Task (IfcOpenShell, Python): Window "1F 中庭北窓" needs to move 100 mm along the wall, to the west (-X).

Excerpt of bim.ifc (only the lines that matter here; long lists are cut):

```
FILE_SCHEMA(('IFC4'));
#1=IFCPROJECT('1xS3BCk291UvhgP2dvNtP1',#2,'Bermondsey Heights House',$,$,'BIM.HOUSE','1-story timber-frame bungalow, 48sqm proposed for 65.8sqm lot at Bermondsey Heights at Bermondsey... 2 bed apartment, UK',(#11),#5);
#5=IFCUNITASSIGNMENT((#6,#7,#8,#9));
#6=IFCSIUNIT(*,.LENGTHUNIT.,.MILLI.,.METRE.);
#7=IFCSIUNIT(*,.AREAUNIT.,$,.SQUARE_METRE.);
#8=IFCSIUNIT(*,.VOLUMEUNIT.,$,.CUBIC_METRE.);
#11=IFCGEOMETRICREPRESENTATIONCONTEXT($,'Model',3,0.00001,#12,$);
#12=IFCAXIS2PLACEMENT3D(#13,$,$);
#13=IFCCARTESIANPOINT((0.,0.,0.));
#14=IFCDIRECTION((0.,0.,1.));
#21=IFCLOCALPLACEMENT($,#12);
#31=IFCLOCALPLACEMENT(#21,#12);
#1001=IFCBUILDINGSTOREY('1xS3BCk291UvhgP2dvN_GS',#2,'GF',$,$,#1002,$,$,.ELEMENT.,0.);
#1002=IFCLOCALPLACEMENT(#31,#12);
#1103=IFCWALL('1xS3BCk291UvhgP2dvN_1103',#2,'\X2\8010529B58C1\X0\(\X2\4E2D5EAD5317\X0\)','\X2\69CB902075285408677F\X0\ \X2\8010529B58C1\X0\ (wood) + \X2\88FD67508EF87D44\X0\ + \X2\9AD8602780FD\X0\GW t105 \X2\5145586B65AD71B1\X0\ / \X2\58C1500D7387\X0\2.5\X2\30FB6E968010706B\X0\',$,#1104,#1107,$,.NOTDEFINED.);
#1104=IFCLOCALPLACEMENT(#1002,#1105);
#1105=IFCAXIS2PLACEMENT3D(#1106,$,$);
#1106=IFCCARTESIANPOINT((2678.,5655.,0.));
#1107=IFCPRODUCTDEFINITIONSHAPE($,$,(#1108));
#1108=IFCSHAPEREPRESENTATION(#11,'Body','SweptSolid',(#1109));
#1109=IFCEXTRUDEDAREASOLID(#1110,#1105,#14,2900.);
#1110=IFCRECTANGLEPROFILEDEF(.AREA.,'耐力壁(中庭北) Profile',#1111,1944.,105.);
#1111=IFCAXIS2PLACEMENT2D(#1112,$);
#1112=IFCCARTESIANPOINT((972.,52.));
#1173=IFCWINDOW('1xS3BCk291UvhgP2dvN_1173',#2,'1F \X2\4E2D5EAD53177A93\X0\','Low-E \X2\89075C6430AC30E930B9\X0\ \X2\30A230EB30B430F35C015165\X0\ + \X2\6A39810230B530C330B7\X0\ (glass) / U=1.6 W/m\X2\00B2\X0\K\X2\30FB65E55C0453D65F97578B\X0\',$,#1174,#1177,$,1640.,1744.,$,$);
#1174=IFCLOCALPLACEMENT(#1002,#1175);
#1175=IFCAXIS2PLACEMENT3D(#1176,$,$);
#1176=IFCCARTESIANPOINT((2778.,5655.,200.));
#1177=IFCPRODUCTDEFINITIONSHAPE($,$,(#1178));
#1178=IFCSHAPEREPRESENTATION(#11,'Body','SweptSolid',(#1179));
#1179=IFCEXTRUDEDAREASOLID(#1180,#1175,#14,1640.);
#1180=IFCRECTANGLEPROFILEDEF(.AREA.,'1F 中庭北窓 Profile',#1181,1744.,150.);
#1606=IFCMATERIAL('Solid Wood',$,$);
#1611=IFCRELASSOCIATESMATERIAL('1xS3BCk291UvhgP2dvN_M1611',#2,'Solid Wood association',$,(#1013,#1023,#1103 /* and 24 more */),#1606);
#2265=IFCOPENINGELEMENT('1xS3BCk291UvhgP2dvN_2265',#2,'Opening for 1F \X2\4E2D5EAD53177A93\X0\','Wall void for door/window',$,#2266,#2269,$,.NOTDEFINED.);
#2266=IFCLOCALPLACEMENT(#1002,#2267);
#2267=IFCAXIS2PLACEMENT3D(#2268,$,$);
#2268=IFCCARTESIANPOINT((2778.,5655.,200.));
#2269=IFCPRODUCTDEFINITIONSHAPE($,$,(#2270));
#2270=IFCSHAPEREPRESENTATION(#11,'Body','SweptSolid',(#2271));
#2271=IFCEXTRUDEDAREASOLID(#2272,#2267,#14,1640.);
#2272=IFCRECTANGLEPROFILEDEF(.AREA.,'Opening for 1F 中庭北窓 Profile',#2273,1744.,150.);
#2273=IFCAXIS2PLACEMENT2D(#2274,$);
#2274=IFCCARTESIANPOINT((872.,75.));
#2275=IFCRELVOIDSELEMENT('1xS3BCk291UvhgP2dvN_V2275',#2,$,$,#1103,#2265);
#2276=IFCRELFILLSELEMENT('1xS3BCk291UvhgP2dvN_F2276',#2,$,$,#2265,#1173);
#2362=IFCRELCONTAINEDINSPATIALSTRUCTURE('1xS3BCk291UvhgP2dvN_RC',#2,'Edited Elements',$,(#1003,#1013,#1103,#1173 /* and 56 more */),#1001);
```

```python
import ifcopenshell
import ifcopenshell.api.geometry
import ifcopenshell.util.placement

model = ifcopenshell.open("bim.ifc")

window = model.by_id(1173)
opening = window.FillsVoids[0].RelatingOpeningElement
wall = opening.VoidsElements[0].RelatingBuildingElement

wall_matrix = ifcopenshell.util.placement.get_local_placement(wall.ObjectPlacement)
shift = wall_matrix[:3, 0] * -100.0
before = ifcopenshell.util.placement.get_local_placement(window.ObjectPlacement)[:3, 3].copy()

# The window is not placed relative to its opening, so move both.
for product in (opening, window):
    matrix = ifcopenshell.util.placement.get_local_placement(product.ObjectPlacement)
    matrix[:3, 3] += shift
    ifcopenshell.api.geometry.edit_object_placement(model, product=product, matrix=matrix, is_si=False)

after = ifcopenshell.util.placement.get_local_placement(window.ObjectPlacement)[:3, 3]
print("window moved by", (after - before).round(3) + 0.0)

model.write("bim_rev.ifc")
```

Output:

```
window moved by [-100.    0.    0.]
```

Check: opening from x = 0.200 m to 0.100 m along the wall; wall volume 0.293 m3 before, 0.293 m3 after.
